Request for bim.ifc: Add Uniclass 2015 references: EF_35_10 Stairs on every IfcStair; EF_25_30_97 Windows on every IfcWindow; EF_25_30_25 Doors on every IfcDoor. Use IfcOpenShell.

First a look at what the model holds.

```python
import ifcopenshell

model = ifcopenshell.open("bim.ifc")
print(model.schema)
print("classifications:", [c.Name for c in model.by_type("IfcClassification")])
for ifc_class in ("IfcDoor", "IfcRoof", "IfcStair", "IfcWall", "IfcWindow"):
    print(ifc_class, len(model.by_type(ifc_class)))
```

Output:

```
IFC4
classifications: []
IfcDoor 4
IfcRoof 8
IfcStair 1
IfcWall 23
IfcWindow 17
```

```python
import ifcopenshell
import ifcopenshell.api.classification

model = ifcopenshell.open("bim.ifc")

system = ifcopenshell.api.classification.add_classification(model, classification="Uniclass 2015")

codes = {
    "IfcStair": ("EF_35_10", "Stairs"),
    "IfcWindow": ("EF_25_30_97", "Windows"),
    "IfcDoor": ("EF_25_30_25", "Doors"),
}
for ifc_class, (code, name) in codes.items():
    products = model.by_type(ifc_class)
    ifcopenshell.api.classification.add_reference(
        model, products=products, classification=system, identification=code, name=name
    )
    print(code, len(products))

model.write("bim-out.ifc")
```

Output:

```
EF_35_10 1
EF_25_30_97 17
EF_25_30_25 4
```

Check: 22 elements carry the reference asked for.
